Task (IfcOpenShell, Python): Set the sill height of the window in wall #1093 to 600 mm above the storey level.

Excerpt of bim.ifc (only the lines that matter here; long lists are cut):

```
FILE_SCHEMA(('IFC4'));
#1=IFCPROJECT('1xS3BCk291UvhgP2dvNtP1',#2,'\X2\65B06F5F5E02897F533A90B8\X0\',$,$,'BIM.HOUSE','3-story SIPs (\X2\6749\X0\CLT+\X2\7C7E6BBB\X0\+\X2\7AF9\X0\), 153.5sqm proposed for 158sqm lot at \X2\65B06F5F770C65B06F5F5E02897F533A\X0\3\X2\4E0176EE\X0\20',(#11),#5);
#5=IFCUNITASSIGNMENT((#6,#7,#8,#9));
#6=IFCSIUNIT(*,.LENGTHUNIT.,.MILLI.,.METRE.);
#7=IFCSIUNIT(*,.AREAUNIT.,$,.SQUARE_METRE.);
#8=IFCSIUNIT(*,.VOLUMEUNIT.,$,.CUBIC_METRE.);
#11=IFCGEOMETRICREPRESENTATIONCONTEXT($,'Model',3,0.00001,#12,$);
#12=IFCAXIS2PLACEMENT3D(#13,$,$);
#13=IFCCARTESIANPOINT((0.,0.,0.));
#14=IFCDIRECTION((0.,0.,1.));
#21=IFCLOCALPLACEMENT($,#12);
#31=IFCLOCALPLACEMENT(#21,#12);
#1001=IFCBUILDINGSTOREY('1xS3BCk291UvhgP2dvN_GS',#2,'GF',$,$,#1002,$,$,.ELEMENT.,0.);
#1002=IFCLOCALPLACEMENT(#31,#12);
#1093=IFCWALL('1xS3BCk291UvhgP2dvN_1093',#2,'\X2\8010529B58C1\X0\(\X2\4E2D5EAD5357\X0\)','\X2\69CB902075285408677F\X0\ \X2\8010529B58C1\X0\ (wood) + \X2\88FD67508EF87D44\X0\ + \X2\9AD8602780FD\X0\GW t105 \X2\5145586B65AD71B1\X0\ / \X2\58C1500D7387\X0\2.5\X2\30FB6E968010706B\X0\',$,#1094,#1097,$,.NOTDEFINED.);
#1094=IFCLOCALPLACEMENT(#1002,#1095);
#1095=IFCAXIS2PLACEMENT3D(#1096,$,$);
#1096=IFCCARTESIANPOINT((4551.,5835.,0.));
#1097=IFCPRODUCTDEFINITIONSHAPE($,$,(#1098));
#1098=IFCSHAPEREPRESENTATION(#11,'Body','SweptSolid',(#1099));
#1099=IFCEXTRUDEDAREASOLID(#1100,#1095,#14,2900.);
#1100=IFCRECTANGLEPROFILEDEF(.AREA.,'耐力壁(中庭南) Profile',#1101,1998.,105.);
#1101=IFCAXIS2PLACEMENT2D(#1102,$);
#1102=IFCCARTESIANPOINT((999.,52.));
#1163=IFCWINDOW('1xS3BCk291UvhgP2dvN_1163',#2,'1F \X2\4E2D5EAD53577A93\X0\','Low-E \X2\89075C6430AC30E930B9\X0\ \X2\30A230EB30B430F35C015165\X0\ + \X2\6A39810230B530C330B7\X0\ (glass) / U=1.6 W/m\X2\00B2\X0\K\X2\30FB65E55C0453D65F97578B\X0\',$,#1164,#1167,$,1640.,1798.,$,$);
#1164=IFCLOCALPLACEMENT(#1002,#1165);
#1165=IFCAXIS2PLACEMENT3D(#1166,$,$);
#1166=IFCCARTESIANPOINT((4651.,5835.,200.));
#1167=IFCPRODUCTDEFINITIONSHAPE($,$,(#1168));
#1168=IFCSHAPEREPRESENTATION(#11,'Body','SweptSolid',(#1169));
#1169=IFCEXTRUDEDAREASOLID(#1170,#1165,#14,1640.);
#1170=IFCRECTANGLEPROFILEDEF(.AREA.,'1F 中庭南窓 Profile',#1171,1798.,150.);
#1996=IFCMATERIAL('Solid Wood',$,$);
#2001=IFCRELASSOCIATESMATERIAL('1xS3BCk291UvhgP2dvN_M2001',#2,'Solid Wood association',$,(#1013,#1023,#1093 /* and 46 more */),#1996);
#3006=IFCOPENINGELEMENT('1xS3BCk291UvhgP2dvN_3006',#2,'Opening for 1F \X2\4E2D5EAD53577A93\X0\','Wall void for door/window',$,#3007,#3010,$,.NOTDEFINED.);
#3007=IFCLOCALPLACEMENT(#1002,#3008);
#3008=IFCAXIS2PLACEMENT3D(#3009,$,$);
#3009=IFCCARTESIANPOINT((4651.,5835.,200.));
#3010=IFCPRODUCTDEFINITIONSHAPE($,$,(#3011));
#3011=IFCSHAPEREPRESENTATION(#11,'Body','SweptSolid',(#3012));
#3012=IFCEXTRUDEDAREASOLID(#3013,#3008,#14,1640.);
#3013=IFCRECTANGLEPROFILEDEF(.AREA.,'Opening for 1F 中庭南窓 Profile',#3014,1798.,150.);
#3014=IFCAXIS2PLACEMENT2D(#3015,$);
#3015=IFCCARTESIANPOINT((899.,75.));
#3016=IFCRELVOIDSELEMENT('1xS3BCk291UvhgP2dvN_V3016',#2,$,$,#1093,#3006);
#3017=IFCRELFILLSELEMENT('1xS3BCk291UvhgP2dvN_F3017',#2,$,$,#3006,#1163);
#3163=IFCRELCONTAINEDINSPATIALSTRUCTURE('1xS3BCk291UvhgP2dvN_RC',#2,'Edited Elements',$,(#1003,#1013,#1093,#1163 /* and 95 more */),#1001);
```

```python
import numpy as np
import ifcopenshell
import ifcopenshell.api.geometry
import ifcopenshell.geom
import ifcopenshell.util.element
import ifcopenshell.util.placement
import ifcopenshell.util.shape
import ifcopenshell.util.unit

model = ifcopenshell.open("bim.ifc")
unit_scale = ifcopenshell.util.unit.calculate_unit_scale(model)

window = model.by_guid("1xS3BCk291UvhgP2dvN_1163")
opening = window.FillsVoids[0].RelatingOpeningElement
storey = ifcopenshell.util.element.get_container(window, ifc_class="IfcBuildingStorey")
level = ifcopenshell.util.placement.get_local_placement(storey.ObjectPlacement)[2, 3]

# The opening's origin need not be at the sill, so measure its lowest point.
shape = ifcopenshell.geom.create_shape(ifcopenshell.geom.settings(), opening)
bottom = ifcopenshell.util.shape.get_shape_bottom_elevation(shape, shape.geometry) / unit_scale
dz = level + 600.0 - bottom

shift = np.array([0.0, 0.0, dz])
# The window is not placed relative to its opening, so move both.
for product in (opening, window):
    matrix = ifcopenshell.util.placement.get_local_placement(product.ObjectPlacement)
    matrix[:3, 3] += shift
    ifcopenshell.api.geometry.edit_object_placement(model, product=product, matrix=matrix, is_si=False)

print(f"moved by {dz * unit_scale:+.3f} m")

model.write("bim_rev.ifc")
```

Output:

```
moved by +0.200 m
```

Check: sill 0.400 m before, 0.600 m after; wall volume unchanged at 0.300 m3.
